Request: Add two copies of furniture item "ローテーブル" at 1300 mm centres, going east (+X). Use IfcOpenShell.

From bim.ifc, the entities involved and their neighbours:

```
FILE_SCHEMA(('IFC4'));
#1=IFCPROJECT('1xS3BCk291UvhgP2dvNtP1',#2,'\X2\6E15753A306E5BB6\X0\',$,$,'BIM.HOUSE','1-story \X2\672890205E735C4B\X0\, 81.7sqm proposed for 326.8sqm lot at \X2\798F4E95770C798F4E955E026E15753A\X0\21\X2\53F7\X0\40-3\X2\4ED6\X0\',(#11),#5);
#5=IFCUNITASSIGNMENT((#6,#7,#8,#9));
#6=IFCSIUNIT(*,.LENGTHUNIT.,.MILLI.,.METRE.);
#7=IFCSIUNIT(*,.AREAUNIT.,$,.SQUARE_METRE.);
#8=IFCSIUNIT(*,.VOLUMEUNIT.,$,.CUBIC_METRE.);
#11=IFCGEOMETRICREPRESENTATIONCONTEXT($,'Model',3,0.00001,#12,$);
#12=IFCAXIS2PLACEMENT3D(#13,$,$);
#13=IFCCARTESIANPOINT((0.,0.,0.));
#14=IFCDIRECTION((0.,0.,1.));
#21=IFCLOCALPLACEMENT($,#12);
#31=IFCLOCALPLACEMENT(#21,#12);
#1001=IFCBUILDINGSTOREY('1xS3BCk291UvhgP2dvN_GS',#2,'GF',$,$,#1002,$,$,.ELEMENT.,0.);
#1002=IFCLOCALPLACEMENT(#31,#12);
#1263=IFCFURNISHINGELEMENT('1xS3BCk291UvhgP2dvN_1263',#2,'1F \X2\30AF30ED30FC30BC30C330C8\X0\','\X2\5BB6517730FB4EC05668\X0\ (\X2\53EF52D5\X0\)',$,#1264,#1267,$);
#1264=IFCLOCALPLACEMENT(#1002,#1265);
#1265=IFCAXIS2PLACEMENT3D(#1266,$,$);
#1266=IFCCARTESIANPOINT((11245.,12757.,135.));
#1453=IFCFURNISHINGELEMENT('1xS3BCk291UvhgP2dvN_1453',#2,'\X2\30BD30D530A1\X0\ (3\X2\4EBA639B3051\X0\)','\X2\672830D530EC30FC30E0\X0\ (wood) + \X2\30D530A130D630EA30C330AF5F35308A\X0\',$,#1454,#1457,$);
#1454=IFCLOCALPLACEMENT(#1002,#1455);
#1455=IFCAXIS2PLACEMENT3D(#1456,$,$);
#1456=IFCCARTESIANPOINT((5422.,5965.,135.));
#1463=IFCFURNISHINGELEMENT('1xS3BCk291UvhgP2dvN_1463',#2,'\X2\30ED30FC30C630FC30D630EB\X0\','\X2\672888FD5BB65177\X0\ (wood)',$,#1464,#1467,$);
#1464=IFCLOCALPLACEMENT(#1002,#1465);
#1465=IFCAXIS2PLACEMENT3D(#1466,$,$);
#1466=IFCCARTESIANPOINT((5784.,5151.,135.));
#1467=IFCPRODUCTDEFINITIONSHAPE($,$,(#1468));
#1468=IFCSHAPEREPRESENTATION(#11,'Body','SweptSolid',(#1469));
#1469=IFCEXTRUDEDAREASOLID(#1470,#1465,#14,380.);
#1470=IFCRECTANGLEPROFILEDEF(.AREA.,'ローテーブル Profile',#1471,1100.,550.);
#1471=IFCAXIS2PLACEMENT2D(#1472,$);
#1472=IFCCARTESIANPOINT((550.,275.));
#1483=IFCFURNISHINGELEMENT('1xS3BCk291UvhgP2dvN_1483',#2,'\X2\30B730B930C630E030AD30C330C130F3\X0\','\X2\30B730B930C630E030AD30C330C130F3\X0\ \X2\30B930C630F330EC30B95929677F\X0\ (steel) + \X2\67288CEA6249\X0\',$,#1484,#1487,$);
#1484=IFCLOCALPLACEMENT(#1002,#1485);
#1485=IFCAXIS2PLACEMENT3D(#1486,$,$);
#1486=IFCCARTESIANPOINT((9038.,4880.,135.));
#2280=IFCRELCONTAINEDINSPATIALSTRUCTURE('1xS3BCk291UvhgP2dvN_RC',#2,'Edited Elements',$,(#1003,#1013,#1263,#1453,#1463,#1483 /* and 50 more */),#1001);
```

```python
import numpy as np
import ifcopenshell
import ifcopenshell.api.geometry
import ifcopenshell.api.root
import ifcopenshell.util.element
import ifcopenshell.util.placement
import ifcopenshell.util.unit

model = ifcopenshell.open("bim.ifc")
unit_scale = ifcopenshell.util.unit.calculate_unit_scale(model)


def reuse_history(source, copy):
    """copy_class also copies each property set's owner history, people and application; keep the originals."""
    for rel in copy.IsDefinedBy:
        if rel.is_a("IfcRelDefinesByProperties") and (history := rel.RelatingPropertyDefinition.OwnerHistory):
            rel.RelatingPropertyDefinition.OwnerHistory = source.OwnerHistory
            ifcopenshell.util.element.remove_deep2(model, history)


source = model.by_guid("1xS3BCk291UvhgP2dvN_1463")
base = ifcopenshell.util.placement.get_local_placement(source.ObjectPlacement)
step = np.array([1.0, 0.0, 0.0]) * 1.3 / unit_scale

for i in range(1, 3):
    copy = ifcopenshell.api.root.copy_class(model, product=source)
    copy.Representation = ifcopenshell.util.element.copy_deep(
        model, source.Representation, exclude=["IfcGeometricRepresentationContext", "IfcRepresentationMap"]
    )
    reuse_history(source, copy)
    matrix = base.copy()
    matrix[:3, 3] += i * step
    print("added at", matrix[:3, 3].round(3) + 0.0)
    ifcopenshell.api.geometry.edit_object_placement(model, product=copy, matrix=matrix, is_si=False)

model.write("bim_updated.ifc")
```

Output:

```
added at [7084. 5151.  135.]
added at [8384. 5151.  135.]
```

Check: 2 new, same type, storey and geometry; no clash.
